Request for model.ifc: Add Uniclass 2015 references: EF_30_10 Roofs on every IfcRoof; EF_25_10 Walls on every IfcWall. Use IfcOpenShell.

First a look at what the model holds.

```python
import ifcopenshell

model = ifcopenshell.open("model.ifc")
print(model.schema)
print("classifications:", [c.Name for c in model.by_type("IfcClassification")])
for ifc_class in ("IfcDoor", "IfcRoof", "IfcStair", "IfcWall", "IfcWindow"):
    print(ifc_class, len(model.by_type(ifc_class)))
```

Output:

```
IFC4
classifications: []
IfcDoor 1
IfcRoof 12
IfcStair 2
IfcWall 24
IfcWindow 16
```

```python
import ifcopenshell
import ifcopenshell.api.classification

model = ifcopenshell.open("model.ifc")

system = ifcopenshell.api.classification.add_classification(model, classification="Uniclass 2015")

codes = {
    "IfcRoof": ("EF_30_10", "Roofs"),
    "IfcWall": ("EF_25_10", "Walls"),
}
for ifc_class, (code, name) in codes.items():
    products = model.by_type(ifc_class)
    ifcopenshell.api.classification.add_reference(
        model, products=products, classification=system, identification=code, name=name
    )
    print(code, len(products))

model.write("model_v2.ifc")
```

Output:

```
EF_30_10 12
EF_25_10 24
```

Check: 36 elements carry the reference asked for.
